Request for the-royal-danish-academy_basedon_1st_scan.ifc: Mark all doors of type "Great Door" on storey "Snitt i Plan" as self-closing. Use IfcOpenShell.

First a look at what the model holds.

```python
import ifcopenshell
import ifcopenshell.util.element

model = ifcopenshell.open("the-royal-danish-academy_basedon_1st_scan.ifc")
print(model.schema)
storey = next(s for s in model.by_type("IfcBuildingStorey") if s.Name == "Snitt i Plan")
doors = [e for e in ifcopenshell.util.element.get_decomposition(storey) if e.is_a("IfcDoor")]
seen = {}
for e in doors:
    element_type = ifcopenshell.util.element.get_type(e)
    key = (element_type.Name if element_type != e and element_type else None, ifcopenshell.util.element.get_pset(e, "Pset_DoorCommon", "SelfClosing"))
    seen[key] = seen.get(key, 0) + 1
for (name, value), count in sorted(seen.items(), key=str):
    print(count, "x", name, "|", value)
```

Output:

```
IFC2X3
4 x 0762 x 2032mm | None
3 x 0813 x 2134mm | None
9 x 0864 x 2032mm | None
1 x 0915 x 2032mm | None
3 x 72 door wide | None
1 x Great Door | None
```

```python
import ifcopenshell
import ifcopenshell.api.pset
import ifcopenshell.util.element

model = ifcopenshell.open("the-royal-danish-academy_basedon_1st_scan.ifc")

storey = next(s for s in model.by_type("IfcBuildingStorey") if s.Name == "Snitt i Plan")
doors = [e for e in ifcopenshell.util.element.get_decomposition(storey) if e.is_a("IfcDoor")]

count = 0
for e in doors:
    element_type = ifcopenshell.util.element.get_type(e)
    if element_type in (None, e) or element_type.Name != "Great Door":
        continue
    # add_pset returns the element's existing set when there is one.
    pset = ifcopenshell.api.pset.add_pset(model, product=e, name="Pset_DoorCommon")
    ifcopenshell.api.pset.edit_pset(model, pset=pset, properties={"SelfClosing": True})
    count += 1

print(count, "doors updated")

model.write("the-royal-danish-academy_basedon_1st_scan_rev.ifc")
```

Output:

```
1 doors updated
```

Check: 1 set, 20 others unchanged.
